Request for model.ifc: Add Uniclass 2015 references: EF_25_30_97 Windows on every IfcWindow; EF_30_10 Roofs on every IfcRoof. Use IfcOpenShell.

First a look at what the model holds.

```python
import ifcopenshell

model = ifcopenshell.open("model.ifc")
print(model.schema)
print("classifications:", [c.Name for c in model.by_type("IfcClassification")])
for ifc_class in ("IfcDoor", "IfcRoof", "IfcStair", "IfcWall", "IfcWindow"):
    print(ifc_class, len(model.by_type(ifc_class)))
```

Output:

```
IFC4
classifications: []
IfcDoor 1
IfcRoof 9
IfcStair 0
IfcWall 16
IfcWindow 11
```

```python
import ifcopenshell
import ifcopenshell.api.classification

model = ifcopenshell.open("model.ifc")

system = ifcopenshell.api.classification.add_classification(model, classification="Uniclass 2015")

codes = {
    "IfcWindow": ("EF_25_30_97", "Windows"),
    "IfcRoof": ("EF_30_10", "Roofs"),
}
for ifc_class, (code, name) in codes.items():
    products = model.by_type(ifc_class)
    ifcopenshell.api.classification.add_reference(
        model, products=products, classification=system, identification=code, name=name
    )
    print(code, len(products))

model.write("model_rev.ifc")
```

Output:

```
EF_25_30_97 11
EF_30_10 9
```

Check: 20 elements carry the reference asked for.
